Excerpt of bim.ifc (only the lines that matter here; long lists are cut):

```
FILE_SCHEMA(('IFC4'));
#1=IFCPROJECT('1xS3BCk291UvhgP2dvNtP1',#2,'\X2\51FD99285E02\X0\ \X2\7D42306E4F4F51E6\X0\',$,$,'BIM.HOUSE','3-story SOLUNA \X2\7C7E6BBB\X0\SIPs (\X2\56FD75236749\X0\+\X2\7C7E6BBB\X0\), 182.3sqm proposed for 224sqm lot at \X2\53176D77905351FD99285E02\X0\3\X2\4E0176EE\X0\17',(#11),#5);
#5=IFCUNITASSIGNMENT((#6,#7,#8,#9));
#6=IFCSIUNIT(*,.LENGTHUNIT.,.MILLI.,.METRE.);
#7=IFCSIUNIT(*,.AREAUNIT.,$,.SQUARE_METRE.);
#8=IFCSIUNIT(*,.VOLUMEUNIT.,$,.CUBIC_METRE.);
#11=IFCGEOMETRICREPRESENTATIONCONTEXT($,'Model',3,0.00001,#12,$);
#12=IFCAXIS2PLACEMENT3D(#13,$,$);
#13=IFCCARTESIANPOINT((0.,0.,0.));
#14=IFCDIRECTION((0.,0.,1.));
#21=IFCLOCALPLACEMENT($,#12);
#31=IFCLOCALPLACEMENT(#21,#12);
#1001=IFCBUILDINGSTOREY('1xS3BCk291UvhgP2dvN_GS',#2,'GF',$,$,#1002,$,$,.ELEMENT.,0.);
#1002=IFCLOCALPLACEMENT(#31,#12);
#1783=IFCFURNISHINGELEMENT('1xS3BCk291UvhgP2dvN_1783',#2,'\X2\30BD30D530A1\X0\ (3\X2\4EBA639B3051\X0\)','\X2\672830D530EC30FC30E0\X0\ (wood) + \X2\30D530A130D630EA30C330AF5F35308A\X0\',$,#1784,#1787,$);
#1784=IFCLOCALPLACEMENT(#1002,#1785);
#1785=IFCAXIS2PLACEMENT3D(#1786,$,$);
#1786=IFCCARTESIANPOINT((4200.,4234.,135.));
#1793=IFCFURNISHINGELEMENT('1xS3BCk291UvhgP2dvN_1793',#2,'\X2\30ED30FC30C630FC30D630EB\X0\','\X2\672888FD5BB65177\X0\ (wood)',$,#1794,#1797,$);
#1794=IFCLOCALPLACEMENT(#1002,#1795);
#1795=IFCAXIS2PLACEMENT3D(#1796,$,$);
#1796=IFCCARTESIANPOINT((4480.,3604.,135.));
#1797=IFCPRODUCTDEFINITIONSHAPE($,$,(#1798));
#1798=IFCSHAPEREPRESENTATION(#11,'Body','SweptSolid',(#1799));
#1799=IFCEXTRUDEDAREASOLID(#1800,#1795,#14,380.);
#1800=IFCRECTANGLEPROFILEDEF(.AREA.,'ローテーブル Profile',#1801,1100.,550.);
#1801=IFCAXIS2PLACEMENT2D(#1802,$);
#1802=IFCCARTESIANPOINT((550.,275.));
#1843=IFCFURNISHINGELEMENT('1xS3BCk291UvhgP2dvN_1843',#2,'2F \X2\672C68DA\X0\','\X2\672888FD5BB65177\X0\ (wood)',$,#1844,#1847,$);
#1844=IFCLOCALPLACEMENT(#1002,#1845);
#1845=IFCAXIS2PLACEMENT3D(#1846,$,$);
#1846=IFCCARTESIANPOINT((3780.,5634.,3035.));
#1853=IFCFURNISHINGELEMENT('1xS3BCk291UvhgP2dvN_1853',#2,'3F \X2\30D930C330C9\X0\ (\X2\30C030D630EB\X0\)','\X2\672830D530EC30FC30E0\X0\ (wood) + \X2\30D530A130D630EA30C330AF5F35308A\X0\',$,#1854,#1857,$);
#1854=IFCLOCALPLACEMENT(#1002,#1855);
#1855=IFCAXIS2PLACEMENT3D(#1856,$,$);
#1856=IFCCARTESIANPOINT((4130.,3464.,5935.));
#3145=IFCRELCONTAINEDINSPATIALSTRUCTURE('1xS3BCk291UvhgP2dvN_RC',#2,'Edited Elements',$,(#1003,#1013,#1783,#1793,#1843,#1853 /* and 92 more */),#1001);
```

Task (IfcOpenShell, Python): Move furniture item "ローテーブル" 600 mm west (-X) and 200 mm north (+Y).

```python
import ifcopenshell
import ifcopenshell.api.geometry
import ifcopenshell.util.placement
import ifcopenshell.util.unit

model = ifcopenshell.open("bim.ifc")
unit_scale = ifcopenshell.util.unit.calculate_unit_scale(model)

item = model.by_guid("1xS3BCk291UvhgP2dvN_1793")
matrix = ifcopenshell.util.placement.get_local_placement(item.ObjectPlacement)
matrix[0, 3] -= 0.6 / unit_scale
matrix[1, 3] += 0.2 / unit_scale
ifcopenshell.api.geometry.edit_object_placement(model, product=item, matrix=matrix, is_si=False)

print(ifcopenshell.util.placement.get_local_placement(item.ObjectPlacement).round(3) + 0.0)

model.write("bim_rev.ifc")
```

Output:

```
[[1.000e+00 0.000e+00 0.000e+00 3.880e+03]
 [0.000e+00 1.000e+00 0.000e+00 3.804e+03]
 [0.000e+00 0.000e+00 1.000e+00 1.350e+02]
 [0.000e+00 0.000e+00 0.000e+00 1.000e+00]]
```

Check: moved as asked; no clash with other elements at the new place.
